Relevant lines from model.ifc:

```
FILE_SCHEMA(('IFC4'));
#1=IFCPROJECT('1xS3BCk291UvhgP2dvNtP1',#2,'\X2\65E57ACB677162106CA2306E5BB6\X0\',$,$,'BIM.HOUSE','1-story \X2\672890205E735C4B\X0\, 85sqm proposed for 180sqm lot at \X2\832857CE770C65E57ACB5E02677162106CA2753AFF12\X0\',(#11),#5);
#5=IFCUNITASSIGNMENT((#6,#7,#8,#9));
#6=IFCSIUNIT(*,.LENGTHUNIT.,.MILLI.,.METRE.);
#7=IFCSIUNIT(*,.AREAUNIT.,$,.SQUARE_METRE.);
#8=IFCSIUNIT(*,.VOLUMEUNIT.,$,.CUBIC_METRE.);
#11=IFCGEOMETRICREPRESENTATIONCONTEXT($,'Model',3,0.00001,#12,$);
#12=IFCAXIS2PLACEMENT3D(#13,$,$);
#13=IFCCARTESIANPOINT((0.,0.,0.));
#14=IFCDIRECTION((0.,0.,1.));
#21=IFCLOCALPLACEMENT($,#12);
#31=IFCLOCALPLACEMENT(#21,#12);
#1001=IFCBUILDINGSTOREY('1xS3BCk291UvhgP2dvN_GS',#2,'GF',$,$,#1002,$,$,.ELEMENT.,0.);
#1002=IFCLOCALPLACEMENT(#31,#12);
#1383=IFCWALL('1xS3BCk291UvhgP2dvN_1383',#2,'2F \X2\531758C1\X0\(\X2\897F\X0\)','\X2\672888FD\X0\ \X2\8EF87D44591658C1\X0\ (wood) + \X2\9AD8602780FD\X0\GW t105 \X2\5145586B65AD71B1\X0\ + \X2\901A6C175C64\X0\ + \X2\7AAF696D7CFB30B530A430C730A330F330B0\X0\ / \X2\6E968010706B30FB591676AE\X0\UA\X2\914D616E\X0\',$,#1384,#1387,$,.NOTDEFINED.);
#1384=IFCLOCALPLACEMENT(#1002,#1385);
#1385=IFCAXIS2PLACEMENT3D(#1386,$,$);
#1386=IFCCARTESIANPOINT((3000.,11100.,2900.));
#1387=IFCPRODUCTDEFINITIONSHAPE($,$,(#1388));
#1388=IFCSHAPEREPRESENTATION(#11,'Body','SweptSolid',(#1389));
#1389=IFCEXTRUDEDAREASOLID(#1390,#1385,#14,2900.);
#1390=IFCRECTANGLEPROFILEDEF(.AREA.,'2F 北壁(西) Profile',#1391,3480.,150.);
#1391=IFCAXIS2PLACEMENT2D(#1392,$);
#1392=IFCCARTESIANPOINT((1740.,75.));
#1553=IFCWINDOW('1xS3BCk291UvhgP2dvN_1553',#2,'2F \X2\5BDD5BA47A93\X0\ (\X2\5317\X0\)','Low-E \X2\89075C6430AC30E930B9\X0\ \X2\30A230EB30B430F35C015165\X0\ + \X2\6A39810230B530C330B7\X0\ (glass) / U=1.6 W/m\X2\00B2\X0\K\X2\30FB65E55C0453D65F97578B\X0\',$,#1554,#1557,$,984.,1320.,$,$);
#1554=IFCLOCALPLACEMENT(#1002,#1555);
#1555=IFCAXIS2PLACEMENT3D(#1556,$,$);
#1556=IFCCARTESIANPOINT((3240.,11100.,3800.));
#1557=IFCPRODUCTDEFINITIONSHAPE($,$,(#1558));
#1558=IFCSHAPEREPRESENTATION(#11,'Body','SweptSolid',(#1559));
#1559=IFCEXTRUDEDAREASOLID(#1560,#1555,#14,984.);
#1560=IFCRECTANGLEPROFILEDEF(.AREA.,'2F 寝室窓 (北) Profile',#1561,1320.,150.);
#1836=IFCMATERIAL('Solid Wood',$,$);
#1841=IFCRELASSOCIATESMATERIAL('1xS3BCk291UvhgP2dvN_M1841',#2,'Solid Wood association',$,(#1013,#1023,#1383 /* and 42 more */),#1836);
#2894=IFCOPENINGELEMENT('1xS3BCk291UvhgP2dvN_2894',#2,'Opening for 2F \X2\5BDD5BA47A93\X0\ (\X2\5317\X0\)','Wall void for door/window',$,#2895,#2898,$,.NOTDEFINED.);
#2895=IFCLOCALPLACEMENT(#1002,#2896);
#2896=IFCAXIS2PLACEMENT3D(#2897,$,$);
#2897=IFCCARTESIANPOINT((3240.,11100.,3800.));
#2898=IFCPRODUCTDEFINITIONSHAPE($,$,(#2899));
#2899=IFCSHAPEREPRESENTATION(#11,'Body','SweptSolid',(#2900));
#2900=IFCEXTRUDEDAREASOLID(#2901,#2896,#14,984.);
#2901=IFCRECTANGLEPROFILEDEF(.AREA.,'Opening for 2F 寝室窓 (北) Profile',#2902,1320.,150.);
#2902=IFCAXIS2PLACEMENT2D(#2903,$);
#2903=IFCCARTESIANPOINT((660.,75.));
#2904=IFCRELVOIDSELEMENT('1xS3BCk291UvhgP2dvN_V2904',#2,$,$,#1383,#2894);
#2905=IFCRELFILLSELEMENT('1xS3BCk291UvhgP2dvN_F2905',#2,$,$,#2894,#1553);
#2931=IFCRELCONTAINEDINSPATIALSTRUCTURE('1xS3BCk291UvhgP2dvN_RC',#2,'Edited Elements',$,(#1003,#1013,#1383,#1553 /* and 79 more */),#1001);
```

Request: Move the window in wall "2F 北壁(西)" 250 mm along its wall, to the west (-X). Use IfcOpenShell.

```python
import ifcopenshell
import ifcopenshell.api.geometry
import ifcopenshell.util.placement

model = ifcopenshell.open("model.ifc")

window = model.by_guid("1xS3BCk291UvhgP2dvN_1553")
opening = window.FillsVoids[0].RelatingOpeningElement
wall = opening.VoidsElements[0].RelatingBuildingElement

wall_matrix = ifcopenshell.util.placement.get_local_placement(wall.ObjectPlacement)
shift = wall_matrix[:3, 0] * -250.0
before = ifcopenshell.util.placement.get_local_placement(window.ObjectPlacement)[:3, 3].copy()

# The window is not placed relative to its opening, so move both.
for product in (opening, window):
    matrix = ifcopenshell.util.placement.get_local_placement(product.ObjectPlacement)
    matrix[:3, 3] += shift
    ifcopenshell.api.geometry.edit_object_placement(model, product=product, matrix=matrix, is_si=False)

after = ifcopenshell.util.placement.get_local_placement(window.ObjectPlacement)[:3, 3]
print("window moved by", (after - before).round(3) + 0.0)

model.write("model-out.ifc")
```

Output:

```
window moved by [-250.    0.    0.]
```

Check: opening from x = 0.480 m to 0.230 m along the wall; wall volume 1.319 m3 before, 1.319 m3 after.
